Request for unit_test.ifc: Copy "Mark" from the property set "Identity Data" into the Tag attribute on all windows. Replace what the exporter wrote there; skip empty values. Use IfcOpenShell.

First a look at what the model holds.

```python
import ifcopenshell
import ifcopenshell.util.element

model = ifcopenshell.open("unit_test.ifc")
print(model.schema)
windows = model.by_type("IfcWindow")
print(len(windows), "windows")
for e in windows[:8]:
    source = ifcopenshell.util.element.get_pset(e, "Identity Data", "Mark")
    target = e.Tag
    print(e.id(), repr(source), repr(target), sep=" | ")
```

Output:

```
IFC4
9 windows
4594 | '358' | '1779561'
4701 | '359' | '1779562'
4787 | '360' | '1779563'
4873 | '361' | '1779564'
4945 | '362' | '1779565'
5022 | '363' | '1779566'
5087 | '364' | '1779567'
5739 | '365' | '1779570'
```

```python
import ifcopenshell
import ifcopenshell.util.element

model = ifcopenshell.open("unit_test.ifc")

count = 0
for e in model.by_type("IfcWindow"):
    value = ifcopenshell.util.element.get_pset(e, "Identity Data", "Mark")
    current = e.Tag
    if not value or not value.strip() or current == value:
        continue
    e.Tag = value
    count += 1

print(count, "windows updated")

model.write("unit_test_edited.ifc")
```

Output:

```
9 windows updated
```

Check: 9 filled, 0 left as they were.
